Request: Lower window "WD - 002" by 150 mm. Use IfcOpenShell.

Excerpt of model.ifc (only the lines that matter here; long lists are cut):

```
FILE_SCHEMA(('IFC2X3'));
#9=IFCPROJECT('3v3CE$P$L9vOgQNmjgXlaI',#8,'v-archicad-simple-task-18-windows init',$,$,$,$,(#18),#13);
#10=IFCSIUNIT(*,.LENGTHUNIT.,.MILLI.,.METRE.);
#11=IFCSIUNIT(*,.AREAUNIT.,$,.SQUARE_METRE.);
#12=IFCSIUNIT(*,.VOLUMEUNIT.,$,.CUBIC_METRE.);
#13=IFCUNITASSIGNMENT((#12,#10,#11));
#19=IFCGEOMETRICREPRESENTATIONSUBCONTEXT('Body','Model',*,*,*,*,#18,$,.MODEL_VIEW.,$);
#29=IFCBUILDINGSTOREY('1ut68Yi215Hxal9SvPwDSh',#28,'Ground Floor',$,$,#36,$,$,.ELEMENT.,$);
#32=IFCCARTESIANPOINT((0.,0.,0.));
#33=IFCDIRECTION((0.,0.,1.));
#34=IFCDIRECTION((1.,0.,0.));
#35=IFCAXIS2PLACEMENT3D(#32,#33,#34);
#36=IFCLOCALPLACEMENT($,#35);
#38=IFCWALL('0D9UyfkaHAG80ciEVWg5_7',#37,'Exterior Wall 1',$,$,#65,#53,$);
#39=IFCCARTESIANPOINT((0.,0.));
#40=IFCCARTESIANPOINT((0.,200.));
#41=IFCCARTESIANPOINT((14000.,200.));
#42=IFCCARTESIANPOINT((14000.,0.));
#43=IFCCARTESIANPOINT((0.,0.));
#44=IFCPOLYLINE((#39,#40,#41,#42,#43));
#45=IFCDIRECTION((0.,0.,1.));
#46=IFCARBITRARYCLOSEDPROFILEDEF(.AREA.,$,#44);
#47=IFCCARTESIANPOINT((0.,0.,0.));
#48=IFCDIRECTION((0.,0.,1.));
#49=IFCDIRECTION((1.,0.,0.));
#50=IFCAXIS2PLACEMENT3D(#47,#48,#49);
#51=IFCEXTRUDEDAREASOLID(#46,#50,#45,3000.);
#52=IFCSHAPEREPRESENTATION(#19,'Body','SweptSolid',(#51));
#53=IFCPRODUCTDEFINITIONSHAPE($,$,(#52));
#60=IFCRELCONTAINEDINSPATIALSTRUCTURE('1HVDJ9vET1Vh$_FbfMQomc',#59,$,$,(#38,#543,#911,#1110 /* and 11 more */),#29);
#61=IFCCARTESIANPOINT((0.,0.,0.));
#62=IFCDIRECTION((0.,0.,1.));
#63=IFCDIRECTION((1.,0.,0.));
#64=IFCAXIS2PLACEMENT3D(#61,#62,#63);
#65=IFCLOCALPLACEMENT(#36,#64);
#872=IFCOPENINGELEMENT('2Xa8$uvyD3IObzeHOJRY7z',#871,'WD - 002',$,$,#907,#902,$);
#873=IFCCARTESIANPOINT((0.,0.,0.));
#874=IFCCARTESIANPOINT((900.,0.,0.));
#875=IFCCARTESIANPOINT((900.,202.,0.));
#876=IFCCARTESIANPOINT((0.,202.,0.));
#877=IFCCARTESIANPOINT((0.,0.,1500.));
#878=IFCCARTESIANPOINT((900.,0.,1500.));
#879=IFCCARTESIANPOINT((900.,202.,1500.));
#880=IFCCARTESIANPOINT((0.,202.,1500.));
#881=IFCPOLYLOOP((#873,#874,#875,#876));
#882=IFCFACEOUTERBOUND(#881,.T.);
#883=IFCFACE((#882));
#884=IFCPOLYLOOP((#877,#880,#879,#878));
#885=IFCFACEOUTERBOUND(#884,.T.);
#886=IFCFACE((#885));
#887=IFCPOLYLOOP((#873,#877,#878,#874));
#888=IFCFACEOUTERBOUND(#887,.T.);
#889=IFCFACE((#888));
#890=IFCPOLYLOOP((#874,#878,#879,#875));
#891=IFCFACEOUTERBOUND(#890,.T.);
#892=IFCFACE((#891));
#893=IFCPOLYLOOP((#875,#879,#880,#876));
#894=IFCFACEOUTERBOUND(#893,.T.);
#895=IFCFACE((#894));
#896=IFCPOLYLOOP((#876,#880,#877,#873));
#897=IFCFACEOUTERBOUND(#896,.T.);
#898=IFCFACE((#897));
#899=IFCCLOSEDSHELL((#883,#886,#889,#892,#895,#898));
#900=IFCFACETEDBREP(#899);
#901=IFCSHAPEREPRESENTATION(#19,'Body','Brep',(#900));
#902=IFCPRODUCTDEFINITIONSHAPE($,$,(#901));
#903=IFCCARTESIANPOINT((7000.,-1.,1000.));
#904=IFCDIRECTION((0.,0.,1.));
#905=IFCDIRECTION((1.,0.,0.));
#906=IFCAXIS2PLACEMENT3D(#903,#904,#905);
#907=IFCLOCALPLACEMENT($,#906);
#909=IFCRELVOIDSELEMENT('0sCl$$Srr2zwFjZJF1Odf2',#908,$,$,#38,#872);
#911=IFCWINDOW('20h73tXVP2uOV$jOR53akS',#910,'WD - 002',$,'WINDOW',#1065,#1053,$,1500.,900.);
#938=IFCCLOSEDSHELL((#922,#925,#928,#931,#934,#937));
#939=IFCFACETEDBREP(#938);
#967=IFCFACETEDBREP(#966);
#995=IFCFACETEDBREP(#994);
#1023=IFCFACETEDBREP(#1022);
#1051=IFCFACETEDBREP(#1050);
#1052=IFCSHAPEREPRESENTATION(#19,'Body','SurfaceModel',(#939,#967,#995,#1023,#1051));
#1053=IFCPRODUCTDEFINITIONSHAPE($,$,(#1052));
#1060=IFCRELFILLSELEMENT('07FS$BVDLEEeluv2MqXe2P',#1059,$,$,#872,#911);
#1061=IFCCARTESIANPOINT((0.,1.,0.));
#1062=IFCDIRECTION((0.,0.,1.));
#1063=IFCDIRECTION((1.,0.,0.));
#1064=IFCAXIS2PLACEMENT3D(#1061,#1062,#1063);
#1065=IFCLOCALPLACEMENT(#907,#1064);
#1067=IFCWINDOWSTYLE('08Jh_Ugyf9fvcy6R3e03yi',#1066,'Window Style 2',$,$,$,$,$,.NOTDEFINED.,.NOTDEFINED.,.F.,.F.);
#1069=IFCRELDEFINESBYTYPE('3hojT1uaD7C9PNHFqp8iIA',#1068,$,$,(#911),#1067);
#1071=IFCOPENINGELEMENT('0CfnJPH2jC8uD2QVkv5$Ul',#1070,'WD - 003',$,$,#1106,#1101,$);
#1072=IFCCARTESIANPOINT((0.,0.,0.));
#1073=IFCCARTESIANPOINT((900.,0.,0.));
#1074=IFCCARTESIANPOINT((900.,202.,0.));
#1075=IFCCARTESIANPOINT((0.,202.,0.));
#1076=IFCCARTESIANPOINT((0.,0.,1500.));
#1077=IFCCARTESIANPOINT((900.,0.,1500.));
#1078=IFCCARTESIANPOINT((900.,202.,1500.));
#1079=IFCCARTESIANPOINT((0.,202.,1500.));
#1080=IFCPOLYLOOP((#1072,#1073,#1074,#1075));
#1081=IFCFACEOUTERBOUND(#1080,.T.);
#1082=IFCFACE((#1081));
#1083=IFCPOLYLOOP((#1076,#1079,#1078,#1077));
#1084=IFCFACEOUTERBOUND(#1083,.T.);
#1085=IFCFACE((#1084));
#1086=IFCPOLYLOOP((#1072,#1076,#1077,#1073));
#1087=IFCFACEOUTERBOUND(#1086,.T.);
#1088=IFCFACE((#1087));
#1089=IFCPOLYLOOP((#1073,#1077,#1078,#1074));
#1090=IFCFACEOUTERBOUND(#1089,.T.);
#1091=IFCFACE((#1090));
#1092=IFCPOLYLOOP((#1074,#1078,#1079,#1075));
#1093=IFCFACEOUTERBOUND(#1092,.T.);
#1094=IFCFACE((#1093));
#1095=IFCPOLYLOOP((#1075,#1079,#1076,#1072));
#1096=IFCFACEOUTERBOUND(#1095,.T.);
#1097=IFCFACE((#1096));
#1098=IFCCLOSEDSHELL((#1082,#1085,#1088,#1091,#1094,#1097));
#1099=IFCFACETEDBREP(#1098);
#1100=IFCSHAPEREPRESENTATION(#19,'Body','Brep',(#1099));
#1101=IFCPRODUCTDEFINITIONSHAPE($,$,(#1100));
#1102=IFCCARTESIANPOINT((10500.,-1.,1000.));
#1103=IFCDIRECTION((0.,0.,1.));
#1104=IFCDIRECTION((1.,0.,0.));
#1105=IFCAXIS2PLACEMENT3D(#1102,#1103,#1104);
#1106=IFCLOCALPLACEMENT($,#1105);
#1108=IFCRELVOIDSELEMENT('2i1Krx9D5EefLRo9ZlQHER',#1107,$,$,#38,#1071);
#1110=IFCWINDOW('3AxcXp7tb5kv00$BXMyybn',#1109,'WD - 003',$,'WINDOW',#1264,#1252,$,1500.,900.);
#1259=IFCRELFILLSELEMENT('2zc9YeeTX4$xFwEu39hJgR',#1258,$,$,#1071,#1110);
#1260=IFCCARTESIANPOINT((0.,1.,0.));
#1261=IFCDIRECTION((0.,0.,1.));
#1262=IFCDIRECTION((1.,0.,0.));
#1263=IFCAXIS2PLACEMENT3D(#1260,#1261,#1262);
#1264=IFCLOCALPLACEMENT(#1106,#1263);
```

```python
import numpy as np
import ifcopenshell
import ifcopenshell.api.geometry
import ifcopenshell.util.placement
import ifcopenshell.util.unit

model = ifcopenshell.open("model.ifc")
unit_scale = ifcopenshell.util.unit.calculate_unit_scale(model)

window = model.by_guid("20h73tXVP2uOV$jOR53akS")
opening = window.FillsVoids[0].RelatingOpeningElement
dz = -150.0

shift = np.array([0.0, 0.0, dz])
# The window is placed relative to its opening, so it follows when the opening moves.
matrix = ifcopenshell.util.placement.get_local_placement(opening.ObjectPlacement)
matrix[:3, 3] += shift
ifcopenshell.api.geometry.edit_object_placement(
    model, product=opening, matrix=matrix, is_si=False, should_transform_children=True
)

print(f"moved by {dz * unit_scale:+.3f} m")

model.write("model_rev.ifc")
```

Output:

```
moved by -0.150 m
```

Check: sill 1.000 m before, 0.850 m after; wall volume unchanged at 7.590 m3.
